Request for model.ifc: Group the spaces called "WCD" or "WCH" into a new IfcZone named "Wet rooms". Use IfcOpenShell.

First a look at what the model holds.

```python
import ifcopenshell

model = ifcopenshell.open("model.ifc")
print(model.schema)
seen = {}
for space in model.by_type("IfcSpace"):
    seen[space.LongName] = seen.get(space.LongName, 0) + 1
for name, count in sorted(seen.items(), key=str):
    print(count, "x", name)
print("zones:", [z.Name for z in model.by_type("IfcZone")][:20])
```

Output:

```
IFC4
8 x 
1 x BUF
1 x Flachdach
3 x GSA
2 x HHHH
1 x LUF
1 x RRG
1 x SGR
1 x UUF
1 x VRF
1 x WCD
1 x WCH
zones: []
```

```python
import ifcopenshell
import ifcopenshell.api.group
import ifcopenshell.api.root

model = ifcopenshell.open("model.ifc")

names = {"WCD", "WCH"}
spaces = [s for s in model.by_type("IfcSpace") if s.LongName in names]

zone = ifcopenshell.api.root.create_entity(model, ifc_class="IfcZone", name="Wet rooms")
ifcopenshell.api.group.assign_group(model, products=spaces, group=zone)
print(len(spaces), "spaces in", zone.Name)

model.write("model_edited.ifc")
```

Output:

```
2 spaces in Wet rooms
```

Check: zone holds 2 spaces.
